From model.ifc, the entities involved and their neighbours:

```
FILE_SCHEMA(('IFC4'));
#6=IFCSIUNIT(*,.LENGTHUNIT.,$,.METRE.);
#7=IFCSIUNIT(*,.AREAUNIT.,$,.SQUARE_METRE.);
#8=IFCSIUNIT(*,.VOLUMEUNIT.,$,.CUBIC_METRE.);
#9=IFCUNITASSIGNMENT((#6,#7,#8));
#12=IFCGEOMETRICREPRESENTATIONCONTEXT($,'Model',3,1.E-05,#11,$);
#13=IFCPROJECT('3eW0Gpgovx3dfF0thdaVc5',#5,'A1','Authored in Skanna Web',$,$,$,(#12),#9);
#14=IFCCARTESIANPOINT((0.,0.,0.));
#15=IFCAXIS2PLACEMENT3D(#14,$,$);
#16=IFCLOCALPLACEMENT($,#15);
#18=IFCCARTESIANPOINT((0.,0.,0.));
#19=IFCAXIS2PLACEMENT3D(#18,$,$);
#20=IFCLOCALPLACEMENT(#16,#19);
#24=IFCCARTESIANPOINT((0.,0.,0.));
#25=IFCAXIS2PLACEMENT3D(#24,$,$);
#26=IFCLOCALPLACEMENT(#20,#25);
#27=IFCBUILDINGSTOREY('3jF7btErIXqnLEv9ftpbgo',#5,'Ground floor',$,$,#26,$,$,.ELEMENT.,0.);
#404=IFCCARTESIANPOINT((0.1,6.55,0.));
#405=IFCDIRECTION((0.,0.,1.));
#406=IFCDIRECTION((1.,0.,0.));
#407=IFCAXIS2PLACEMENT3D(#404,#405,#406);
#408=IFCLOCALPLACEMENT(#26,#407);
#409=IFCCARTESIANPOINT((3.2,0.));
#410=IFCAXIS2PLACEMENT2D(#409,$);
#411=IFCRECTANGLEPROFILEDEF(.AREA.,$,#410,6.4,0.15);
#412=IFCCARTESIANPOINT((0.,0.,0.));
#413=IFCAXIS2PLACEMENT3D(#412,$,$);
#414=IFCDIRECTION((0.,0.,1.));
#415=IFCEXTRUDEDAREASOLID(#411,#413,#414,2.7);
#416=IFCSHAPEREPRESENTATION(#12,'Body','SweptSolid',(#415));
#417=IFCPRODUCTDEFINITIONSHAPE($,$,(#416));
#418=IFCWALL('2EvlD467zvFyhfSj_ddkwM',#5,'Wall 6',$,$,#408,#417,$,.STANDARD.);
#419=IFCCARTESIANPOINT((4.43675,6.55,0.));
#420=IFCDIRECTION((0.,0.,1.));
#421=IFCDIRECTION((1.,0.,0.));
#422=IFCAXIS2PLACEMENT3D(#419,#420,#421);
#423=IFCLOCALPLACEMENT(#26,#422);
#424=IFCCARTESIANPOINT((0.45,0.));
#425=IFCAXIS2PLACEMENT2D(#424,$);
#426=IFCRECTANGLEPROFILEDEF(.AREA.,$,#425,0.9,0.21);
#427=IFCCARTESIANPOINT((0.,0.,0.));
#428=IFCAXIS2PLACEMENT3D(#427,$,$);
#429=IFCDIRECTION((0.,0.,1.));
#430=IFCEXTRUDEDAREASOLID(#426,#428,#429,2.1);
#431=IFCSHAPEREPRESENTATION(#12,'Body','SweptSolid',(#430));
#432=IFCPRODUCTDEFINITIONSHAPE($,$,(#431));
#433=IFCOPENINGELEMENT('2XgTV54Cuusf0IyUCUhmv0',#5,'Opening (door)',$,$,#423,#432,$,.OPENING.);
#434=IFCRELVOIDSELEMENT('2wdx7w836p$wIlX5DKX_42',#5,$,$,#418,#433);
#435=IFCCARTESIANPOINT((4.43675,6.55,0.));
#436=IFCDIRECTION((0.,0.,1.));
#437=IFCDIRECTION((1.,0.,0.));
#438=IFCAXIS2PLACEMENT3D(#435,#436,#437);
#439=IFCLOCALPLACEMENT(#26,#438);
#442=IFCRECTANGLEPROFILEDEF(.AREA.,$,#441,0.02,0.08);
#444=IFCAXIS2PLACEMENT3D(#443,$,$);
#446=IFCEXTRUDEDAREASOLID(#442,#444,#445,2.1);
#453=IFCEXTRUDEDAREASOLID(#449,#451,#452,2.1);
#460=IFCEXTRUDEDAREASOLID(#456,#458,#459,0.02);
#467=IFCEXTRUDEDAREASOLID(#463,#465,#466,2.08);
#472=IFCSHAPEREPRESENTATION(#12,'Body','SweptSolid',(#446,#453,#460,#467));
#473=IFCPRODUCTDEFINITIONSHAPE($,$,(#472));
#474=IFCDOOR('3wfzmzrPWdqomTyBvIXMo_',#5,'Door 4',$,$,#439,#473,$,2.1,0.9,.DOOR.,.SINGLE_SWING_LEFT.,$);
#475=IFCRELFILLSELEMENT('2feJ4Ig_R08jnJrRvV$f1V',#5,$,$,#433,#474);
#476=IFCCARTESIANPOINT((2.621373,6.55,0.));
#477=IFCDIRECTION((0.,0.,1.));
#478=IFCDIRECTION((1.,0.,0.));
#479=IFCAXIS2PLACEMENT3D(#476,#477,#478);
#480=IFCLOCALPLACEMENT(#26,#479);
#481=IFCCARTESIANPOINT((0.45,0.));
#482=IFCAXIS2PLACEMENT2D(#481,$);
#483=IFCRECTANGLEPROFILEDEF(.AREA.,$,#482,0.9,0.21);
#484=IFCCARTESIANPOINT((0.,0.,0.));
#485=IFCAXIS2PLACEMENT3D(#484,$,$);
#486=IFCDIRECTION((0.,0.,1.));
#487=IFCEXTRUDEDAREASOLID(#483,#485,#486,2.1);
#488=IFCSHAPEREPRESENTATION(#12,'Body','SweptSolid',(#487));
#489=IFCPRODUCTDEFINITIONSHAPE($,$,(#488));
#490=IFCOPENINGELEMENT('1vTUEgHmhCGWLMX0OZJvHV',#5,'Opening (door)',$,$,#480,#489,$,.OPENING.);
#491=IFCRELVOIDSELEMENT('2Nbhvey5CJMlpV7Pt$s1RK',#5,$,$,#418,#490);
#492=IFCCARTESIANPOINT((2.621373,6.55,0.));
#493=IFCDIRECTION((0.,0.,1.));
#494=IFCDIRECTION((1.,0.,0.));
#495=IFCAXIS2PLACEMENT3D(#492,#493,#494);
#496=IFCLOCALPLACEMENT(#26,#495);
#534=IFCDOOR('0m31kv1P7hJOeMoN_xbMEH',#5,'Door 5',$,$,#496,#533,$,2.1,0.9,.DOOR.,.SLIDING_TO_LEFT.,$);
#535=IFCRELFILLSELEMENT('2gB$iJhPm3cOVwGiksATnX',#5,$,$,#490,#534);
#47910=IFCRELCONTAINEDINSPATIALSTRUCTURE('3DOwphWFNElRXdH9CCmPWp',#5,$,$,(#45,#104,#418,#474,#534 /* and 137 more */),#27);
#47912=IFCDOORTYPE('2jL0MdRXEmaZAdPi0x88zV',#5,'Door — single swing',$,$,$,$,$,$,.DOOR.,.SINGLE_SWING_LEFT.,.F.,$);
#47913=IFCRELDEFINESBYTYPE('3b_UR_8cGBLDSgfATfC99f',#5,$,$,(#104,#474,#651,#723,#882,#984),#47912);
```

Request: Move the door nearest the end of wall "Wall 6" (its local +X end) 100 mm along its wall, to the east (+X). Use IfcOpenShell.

```python
import ifcopenshell
import ifcopenshell.api.geometry
import ifcopenshell.util.placement
import ifcopenshell.util.unit

model = ifcopenshell.open("model.ifc")
unit_scale = ifcopenshell.util.unit.calculate_unit_scale(model)

door = model.by_id(474)
opening = door.FillsVoids[0].RelatingOpeningElement
wall = opening.VoidsElements[0].RelatingBuildingElement

wall_matrix = ifcopenshell.util.placement.get_local_placement(wall.ObjectPlacement)
shift = wall_matrix[:3, 0] * 0.1 / unit_scale
before = ifcopenshell.util.placement.get_local_placement(door.ObjectPlacement)[:3, 3].copy()

# The door is not placed relative to its opening, so move both.
for product in (opening, door):
    matrix = ifcopenshell.util.placement.get_local_placement(product.ObjectPlacement)
    matrix[:3, 3] += shift
    ifcopenshell.api.geometry.edit_object_placement(model, product=product, matrix=matrix, is_si=False)

after = ifcopenshell.util.placement.get_local_placement(door.ObjectPlacement)[:3, 3]
print("door moved by", (after - before).round(3) + 0.0)

model.write("model_v2.ifc")
```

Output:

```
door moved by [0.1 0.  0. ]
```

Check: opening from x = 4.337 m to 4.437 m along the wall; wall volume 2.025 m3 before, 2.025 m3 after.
